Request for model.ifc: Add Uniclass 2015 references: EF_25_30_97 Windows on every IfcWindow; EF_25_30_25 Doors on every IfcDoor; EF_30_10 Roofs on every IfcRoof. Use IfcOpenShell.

First a look at what the model holds.

```python
import ifcopenshell

model = ifcopenshell.open("model.ifc")
print(model.schema)
print("classifications:", [c.Name for c in model.by_type("IfcClassification")])
for ifc_class in ("IfcDoor", "IfcRoof", "IfcStair", "IfcWall", "IfcWindow"):
    print(ifc_class, len(model.by_type(ifc_class)))
```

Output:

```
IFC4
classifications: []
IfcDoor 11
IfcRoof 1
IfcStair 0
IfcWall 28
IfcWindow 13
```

```python
import ifcopenshell
import ifcopenshell.api.classification

model = ifcopenshell.open("model.ifc")

system = ifcopenshell.api.classification.add_classification(model, classification="Uniclass 2015")

codes = {
    "IfcWindow": ("EF_25_30_97", "Windows"),
    "IfcDoor": ("EF_25_30_25", "Doors"),
    "IfcRoof": ("EF_30_10", "Roofs"),
}
for ifc_class, (code, name) in codes.items():
    products = model.by_type(ifc_class)
    ifcopenshell.api.classification.add_reference(
        model, products=products, classification=system, identification=code, name=name
    )
    print(code, len(products))

model.write("model_v2.ifc")
```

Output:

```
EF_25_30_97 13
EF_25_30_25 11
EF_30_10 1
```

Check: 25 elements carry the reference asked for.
